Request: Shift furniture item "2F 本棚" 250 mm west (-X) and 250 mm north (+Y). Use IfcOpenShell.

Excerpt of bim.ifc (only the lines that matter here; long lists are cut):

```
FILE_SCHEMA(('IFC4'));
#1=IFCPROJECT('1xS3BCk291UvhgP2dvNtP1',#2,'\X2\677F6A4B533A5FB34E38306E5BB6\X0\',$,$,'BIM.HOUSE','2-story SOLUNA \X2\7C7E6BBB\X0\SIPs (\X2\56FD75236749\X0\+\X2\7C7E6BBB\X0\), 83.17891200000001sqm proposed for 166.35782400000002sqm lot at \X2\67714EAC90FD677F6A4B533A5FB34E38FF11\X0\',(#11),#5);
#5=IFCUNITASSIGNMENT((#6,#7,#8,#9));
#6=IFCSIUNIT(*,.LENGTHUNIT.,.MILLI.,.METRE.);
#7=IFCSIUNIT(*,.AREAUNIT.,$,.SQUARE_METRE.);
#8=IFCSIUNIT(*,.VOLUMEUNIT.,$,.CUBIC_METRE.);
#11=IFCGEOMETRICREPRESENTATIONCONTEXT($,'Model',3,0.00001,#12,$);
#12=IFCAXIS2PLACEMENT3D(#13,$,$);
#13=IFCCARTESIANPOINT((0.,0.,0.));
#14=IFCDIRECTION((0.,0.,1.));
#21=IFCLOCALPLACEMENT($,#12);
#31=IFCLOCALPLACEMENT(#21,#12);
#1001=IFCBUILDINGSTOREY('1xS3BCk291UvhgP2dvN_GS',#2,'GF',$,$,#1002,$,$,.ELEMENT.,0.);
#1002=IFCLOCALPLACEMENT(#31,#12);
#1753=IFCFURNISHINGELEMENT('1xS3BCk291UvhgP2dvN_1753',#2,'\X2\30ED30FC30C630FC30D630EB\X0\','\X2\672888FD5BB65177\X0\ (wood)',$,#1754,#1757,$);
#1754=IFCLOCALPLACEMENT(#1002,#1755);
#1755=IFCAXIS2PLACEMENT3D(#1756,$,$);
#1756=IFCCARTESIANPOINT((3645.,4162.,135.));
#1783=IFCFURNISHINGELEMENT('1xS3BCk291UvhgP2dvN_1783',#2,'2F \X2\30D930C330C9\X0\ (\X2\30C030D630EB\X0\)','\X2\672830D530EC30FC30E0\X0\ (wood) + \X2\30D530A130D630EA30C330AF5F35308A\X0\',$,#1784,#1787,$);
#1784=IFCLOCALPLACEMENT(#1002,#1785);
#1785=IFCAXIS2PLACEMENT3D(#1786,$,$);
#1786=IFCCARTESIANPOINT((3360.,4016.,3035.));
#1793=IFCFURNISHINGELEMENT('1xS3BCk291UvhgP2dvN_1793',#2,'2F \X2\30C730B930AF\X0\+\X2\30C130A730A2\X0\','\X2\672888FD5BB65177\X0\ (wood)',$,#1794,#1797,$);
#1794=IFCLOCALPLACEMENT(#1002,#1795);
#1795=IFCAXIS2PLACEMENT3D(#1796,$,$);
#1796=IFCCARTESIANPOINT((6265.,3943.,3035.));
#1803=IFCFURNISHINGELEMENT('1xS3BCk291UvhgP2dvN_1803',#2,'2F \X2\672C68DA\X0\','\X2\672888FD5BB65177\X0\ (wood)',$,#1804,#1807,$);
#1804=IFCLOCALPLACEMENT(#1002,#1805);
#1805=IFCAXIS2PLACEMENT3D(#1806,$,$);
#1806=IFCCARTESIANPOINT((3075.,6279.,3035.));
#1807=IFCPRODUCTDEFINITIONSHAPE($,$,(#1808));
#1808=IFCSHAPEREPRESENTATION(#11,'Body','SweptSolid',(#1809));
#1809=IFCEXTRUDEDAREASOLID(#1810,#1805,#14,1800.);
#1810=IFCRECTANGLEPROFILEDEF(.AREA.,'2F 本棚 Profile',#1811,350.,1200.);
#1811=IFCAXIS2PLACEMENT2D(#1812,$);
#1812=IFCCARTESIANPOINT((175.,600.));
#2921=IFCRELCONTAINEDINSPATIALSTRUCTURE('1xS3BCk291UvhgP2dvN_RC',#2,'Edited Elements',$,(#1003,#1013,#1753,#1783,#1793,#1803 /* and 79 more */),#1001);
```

```python
import ifcopenshell
import ifcopenshell.api.geometry
import ifcopenshell.util.placement

model = ifcopenshell.open("bim.ifc")

item = model.by_id(1803)
matrix = ifcopenshell.util.placement.get_local_placement(item.ObjectPlacement)
matrix[0, 3] -= 250.0
matrix[1, 3] += 250.0
ifcopenshell.api.geometry.edit_object_placement(model, product=item, matrix=matrix, is_si=False)

print(ifcopenshell.util.placement.get_local_placement(item.ObjectPlacement).round(3) + 0.0)

model.write("bim_v2.ifc")
```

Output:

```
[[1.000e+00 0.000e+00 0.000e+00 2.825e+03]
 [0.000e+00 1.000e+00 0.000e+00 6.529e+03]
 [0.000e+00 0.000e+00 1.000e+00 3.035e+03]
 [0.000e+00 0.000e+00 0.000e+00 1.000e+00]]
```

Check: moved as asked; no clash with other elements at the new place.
